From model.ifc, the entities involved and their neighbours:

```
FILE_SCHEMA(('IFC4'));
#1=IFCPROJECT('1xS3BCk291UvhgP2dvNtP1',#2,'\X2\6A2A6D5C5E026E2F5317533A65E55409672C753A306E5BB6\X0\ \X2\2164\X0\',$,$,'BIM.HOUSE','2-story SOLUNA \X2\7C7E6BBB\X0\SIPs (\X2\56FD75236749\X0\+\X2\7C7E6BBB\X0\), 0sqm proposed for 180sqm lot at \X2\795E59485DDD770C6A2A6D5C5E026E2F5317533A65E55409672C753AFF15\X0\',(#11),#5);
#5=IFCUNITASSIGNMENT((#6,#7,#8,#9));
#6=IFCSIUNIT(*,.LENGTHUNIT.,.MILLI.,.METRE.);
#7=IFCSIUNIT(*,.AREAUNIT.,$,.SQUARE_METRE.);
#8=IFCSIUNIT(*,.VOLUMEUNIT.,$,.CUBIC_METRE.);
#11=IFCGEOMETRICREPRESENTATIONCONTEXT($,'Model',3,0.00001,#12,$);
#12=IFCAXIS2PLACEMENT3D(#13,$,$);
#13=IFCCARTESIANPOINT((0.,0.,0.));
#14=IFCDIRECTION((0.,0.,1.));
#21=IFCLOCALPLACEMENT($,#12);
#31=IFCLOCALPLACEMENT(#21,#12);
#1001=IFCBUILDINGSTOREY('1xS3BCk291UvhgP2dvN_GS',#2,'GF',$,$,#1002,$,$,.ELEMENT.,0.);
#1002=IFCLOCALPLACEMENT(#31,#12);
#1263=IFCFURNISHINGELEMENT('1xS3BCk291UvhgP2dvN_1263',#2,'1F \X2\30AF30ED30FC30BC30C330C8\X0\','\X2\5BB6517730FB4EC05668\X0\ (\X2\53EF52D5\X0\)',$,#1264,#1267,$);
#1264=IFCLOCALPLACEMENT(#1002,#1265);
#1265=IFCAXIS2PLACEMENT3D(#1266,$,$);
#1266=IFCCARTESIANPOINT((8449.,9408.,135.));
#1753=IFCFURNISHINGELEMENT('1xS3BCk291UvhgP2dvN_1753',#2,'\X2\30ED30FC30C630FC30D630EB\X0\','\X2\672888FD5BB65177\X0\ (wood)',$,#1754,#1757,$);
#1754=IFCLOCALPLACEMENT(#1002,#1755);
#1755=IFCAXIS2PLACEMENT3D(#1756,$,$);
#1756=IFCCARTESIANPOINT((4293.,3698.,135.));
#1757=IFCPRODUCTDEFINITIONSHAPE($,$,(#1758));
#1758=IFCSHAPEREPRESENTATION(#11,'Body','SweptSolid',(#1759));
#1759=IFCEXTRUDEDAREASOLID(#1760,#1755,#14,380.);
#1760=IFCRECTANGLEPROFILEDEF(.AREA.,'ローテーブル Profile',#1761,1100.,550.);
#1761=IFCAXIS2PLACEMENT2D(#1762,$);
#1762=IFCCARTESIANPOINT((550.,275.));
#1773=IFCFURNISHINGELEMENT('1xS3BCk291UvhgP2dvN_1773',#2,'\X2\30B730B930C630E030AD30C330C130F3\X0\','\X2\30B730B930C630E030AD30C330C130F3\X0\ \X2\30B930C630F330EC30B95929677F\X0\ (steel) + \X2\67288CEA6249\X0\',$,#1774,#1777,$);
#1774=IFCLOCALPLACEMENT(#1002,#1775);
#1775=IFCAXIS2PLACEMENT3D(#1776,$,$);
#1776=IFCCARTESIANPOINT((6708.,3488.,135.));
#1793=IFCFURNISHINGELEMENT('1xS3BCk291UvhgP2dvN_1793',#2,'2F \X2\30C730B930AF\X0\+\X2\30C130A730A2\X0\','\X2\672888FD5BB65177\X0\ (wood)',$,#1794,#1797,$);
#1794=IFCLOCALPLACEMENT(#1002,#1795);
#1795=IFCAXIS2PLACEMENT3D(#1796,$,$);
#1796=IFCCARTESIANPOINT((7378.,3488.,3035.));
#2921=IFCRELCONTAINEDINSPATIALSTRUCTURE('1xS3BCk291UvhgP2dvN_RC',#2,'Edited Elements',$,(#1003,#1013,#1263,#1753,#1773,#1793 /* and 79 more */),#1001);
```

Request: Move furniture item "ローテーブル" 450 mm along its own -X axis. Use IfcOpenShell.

```python
import ifcopenshell
import ifcopenshell.api.geometry
import ifcopenshell.util.placement
import ifcopenshell.util.unit

model = ifcopenshell.open("model.ifc")
unit_scale = ifcopenshell.util.unit.calculate_unit_scale(model)

item = model.by_id(1753)
matrix = ifcopenshell.util.placement.get_local_placement(item.ObjectPlacement)
matrix[:3, 3] -= matrix[:3, 0] * 0.45 / unit_scale
ifcopenshell.api.geometry.edit_object_placement(model, product=item, matrix=matrix, is_si=False)

print(ifcopenshell.util.placement.get_local_placement(item.ObjectPlacement).round(3) + 0.0)

model.write("model_edited.ifc")
```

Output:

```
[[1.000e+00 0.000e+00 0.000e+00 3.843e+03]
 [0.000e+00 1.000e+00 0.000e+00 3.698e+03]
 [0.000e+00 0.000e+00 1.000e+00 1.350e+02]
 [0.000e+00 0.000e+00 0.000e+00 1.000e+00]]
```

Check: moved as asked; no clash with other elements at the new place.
